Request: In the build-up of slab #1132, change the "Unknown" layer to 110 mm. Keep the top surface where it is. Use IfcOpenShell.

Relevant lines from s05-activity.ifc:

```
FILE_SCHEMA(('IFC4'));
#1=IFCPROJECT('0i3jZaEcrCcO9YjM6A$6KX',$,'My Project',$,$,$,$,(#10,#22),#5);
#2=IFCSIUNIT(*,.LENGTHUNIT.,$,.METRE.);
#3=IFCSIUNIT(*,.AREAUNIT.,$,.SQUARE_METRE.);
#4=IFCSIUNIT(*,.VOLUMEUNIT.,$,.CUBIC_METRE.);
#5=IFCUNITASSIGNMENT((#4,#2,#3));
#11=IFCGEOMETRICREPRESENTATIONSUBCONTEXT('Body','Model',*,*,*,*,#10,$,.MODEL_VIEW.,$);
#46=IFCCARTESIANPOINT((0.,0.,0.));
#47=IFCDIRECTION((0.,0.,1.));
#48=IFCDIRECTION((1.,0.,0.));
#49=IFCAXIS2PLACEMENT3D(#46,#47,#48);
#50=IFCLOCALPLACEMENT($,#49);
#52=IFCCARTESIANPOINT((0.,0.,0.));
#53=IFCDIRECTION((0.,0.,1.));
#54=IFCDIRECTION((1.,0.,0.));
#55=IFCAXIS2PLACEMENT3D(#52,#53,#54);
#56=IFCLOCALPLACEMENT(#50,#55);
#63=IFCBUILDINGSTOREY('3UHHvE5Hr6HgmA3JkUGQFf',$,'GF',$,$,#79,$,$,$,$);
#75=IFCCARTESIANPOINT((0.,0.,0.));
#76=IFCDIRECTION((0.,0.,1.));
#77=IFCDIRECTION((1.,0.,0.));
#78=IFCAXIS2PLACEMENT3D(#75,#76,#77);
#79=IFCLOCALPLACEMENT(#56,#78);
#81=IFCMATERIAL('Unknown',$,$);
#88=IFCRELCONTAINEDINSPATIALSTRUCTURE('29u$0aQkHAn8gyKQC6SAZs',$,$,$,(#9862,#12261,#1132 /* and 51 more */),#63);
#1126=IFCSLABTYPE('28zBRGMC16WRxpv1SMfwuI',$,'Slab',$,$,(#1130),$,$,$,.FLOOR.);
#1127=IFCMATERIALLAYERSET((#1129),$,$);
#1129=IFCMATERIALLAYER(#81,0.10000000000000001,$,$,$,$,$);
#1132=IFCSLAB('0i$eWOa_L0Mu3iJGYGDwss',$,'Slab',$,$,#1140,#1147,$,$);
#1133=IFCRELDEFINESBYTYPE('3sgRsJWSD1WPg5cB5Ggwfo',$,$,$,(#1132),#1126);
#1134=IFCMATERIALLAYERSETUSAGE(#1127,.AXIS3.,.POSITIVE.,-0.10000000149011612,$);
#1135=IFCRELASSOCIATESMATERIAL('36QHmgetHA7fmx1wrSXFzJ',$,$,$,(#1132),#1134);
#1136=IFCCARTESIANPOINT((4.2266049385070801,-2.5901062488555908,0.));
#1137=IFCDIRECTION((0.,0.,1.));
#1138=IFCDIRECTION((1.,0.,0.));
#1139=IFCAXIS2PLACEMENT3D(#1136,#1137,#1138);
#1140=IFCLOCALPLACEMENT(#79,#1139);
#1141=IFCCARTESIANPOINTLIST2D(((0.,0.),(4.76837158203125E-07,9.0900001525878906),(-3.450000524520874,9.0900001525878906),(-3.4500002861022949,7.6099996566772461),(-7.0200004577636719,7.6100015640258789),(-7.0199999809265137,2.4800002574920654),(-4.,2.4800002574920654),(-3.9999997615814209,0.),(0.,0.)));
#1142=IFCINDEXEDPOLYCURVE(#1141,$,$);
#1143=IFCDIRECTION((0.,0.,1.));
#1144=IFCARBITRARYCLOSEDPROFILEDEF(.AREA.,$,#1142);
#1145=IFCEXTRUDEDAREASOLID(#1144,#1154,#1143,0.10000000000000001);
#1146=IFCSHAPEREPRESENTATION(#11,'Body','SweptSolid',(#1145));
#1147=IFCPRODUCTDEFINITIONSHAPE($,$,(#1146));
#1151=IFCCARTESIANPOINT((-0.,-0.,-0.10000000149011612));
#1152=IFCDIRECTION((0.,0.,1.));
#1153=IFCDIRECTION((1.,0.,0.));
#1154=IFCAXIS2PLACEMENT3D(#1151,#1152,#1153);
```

```python
import ifcopenshell
import ifcopenshell.util.element
import ifcopenshell.util.representation
import ifcopenshell.util.unit

model = ifcopenshell.open("s05-activity.ifc")
unit_scale = ifcopenshell.util.unit.calculate_unit_scale(model)

layer_set = model.by_id(1127)
layer = next(l for l in layer_set.MaterialLayers if l.Material and l.Material.Name == "Unknown")
change = 0.11 / unit_scale - layer.LayerThickness
layer.LayerThickness += change

# Geometry does not follow the layer set by itself.
slabs = [e for e in ifcopenshell.util.element.get_elements_by_material(model, layer_set) if e.is_a("IfcSlab")]
for slab in sorted(slabs, key=lambda e: e.id()):
    body = ifcopenshell.util.representation.get_representation(slab, "Model", "Body")
    solid = body.Items[0]
    old_depth = solid.Depth
    solid.Depth += change
    # Extruded upwards: lower the start of the extrusion so the top stays.
    x, y, z = solid.Position.Location.Coordinates
    solid.Position.Location = model.createIfcCartesianPoint((x, y, z - change))
    print(slab.id(), f"{old_depth:g} -> {solid.Depth:g}")

# The layers are counted up from the underside, which has moved.
for usage in {ifcopenshell.util.element.get_material(slab) for slab in slabs}:
    usage.OffsetFromReferenceLine -= change

model.write("s05-activity-out.ifc")
```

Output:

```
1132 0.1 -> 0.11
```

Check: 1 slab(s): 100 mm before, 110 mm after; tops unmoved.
